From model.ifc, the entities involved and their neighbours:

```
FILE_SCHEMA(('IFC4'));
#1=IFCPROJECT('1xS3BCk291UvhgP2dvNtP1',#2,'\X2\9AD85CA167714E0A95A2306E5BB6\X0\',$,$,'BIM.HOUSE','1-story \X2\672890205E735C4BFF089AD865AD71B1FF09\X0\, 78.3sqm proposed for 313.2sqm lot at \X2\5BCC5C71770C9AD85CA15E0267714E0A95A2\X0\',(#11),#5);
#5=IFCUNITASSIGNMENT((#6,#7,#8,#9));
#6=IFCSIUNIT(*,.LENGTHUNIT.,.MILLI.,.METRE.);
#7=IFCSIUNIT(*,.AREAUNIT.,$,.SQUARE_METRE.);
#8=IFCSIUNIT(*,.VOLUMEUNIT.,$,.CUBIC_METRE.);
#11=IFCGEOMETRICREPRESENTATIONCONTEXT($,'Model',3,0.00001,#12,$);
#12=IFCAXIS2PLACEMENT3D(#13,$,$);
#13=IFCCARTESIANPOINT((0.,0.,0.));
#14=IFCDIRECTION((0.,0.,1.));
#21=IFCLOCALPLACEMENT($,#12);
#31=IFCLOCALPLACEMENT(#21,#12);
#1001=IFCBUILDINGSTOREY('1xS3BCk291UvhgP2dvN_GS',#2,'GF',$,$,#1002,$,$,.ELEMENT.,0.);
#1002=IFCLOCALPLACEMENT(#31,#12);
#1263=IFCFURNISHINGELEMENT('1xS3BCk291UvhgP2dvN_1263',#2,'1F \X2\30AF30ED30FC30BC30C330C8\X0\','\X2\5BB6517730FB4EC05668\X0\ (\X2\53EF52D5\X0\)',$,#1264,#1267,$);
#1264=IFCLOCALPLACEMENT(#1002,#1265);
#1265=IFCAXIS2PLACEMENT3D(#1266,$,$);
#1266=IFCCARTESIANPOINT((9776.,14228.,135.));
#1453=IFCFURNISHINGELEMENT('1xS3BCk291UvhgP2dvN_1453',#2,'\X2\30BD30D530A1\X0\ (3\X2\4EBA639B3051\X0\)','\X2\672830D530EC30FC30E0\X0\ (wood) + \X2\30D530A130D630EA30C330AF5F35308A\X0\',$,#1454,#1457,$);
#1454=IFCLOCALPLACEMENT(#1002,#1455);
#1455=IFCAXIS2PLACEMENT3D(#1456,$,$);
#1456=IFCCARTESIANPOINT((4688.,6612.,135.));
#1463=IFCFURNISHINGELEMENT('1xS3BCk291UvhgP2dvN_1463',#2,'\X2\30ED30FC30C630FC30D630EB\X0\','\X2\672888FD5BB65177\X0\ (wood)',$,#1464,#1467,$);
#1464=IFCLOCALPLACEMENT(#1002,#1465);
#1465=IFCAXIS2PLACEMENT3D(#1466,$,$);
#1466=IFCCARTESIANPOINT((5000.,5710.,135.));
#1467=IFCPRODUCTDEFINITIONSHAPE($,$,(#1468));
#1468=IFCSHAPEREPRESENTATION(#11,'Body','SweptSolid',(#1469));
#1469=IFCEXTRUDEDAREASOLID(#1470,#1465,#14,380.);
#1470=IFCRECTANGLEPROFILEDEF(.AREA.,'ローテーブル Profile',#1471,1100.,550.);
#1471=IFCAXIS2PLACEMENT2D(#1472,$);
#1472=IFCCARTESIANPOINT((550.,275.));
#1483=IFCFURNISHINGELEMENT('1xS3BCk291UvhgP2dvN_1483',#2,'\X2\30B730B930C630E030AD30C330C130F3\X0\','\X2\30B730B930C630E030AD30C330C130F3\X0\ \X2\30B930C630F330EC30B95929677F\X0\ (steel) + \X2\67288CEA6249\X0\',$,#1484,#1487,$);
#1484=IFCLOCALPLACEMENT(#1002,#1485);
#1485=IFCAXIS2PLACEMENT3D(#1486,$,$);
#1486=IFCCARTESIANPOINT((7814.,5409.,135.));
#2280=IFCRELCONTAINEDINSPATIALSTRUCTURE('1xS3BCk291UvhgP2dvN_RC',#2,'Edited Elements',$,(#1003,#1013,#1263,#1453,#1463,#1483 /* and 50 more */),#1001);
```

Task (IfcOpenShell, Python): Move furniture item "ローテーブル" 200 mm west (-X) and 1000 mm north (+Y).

```python
import ifcopenshell
import ifcopenshell.api.geometry
import ifcopenshell.util.placement
import ifcopenshell.util.unit

model = ifcopenshell.open("model.ifc")
unit_scale = ifcopenshell.util.unit.calculate_unit_scale(model)

item = model.by_guid("1xS3BCk291UvhgP2dvN_1463")
matrix = ifcopenshell.util.placement.get_local_placement(item.ObjectPlacement)
matrix[0, 3] -= 0.2 / unit_scale
matrix[1, 3] += 1 / unit_scale
ifcopenshell.api.geometry.edit_object_placement(model, product=item, matrix=matrix, is_si=False)

print(ifcopenshell.util.placement.get_local_placement(item.ObjectPlacement).round(3) + 0.0)

model.write("model_updated.ifc")
```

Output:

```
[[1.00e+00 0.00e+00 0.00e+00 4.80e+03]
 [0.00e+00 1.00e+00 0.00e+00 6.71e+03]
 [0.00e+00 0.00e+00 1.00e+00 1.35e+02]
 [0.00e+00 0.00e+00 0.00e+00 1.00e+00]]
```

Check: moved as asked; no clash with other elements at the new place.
